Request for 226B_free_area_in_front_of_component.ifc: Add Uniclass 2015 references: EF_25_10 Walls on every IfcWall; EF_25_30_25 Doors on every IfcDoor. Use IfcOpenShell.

First a look at what the model holds.

```python
import ifcopenshell

model = ifcopenshell.open("226B_free_area_in_front_of_component.ifc")
print(model.schema)
print("classifications:", [c.Name for c in model.by_type("IfcClassification")])
for ifc_class in ("IfcDoor", "IfcRoof", "IfcStair", "IfcWall", "IfcWindow"):
    print(ifc_class, len(model.by_type(ifc_class)))
```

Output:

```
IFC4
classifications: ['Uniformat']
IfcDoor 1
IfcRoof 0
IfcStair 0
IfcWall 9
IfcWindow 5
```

```python
import ifcopenshell
import ifcopenshell.api.classification

model = ifcopenshell.open("226B_free_area_in_front_of_component.ifc")

system = ifcopenshell.api.classification.add_classification(model, classification="Uniclass 2015")

codes = {
    "IfcWall": ("EF_25_10", "Walls"),
    "IfcDoor": ("EF_25_30_25", "Doors"),
}
for ifc_class, (code, name) in codes.items():
    products = model.by_type(ifc_class)
    ifcopenshell.api.classification.add_reference(
        model, products=products, classification=system, identification=code, name=name
    )
    print(code, len(products))

model.write("226B_free_area_in_front_of_component-out.ifc")
```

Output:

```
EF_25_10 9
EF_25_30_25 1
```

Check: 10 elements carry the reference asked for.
